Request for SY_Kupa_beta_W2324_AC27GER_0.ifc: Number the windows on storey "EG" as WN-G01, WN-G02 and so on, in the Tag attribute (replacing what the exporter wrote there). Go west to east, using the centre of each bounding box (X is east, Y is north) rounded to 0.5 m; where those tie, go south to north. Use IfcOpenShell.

First a look at what the model holds.

```python
import ifcopenshell
import ifcopenshell.util.element
import ifcopenshell.util.placement

model = ifcopenshell.open("SY_Kupa_beta_W2324_AC27GER_0.ifc")
print(model.schema)
storey = next(s for s in model.by_type("IfcBuildingStorey") if s.Name == "EG")
windows = [e for e in ifcopenshell.util.element.get_decomposition(storey) if e.is_a("IfcWindow")]
for e in sorted(windows, key=lambda e: e.id()):
    origin = ifcopenshell.util.placement.get_local_placement(e.ObjectPlacement)[:3, 3]
    print(e.id(), e.Tag, e.Name, origin.round(2) + 0.0, sep=" | ")
```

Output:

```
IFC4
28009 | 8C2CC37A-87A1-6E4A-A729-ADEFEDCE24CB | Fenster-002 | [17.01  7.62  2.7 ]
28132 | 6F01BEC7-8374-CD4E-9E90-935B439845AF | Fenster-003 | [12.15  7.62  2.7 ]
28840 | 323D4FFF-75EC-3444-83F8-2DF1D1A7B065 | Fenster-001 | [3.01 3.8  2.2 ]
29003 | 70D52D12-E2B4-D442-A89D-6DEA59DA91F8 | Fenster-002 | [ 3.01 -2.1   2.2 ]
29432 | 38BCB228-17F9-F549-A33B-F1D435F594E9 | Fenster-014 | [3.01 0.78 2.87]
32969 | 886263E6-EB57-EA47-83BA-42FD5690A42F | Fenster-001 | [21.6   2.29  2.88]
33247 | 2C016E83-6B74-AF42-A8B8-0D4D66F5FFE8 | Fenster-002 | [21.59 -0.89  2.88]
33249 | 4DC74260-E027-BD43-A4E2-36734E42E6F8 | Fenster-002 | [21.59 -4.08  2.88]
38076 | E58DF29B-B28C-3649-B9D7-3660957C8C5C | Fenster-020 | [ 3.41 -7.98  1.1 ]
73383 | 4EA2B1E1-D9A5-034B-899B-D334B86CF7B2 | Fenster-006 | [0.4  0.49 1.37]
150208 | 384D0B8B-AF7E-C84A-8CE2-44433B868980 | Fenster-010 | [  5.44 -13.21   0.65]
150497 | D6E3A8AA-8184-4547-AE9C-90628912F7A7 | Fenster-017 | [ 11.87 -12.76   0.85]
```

```python
import ifcopenshell
import ifcopenshell.geom
import ifcopenshell.util.element
import ifcopenshell.util.shape

model = ifcopenshell.open("SY_Kupa_beta_W2324_AC27GER_0.ifc")
settings = ifcopenshell.geom.settings()
settings.set("use-world-coords", True)


def centre(element):
    shape = ifcopenshell.geom.create_shape(settings, element)
    return ifcopenshell.util.shape.get_bbox_centroid(shape.geometry)


storey = next(s for s in model.by_type("IfcBuildingStorey") if s.Name == "EG")
windows = [e for e in ifcopenshell.util.element.get_decomposition(storey) if e.is_a("IfcWindow")]

# Insertion points can sit at a corner or the storey origin, so sort by the geometry (in metres).
centres = {e: centre(e) for e in windows}
windows.sort(key=lambda e: (round(centres[e][0] / 0.5), centres[e][1]))

for i, e in enumerate(windows, start=1):
    number = f"WN-G{i:02d}"
    e.Tag = number
    print(e.id(), number)

model.write("SY_Kupa_beta_W2324_AC27GER_0_edited.ifc")
```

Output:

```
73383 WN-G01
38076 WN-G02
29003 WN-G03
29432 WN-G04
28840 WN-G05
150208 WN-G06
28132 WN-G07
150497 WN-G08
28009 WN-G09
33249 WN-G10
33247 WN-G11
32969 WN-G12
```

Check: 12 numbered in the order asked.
